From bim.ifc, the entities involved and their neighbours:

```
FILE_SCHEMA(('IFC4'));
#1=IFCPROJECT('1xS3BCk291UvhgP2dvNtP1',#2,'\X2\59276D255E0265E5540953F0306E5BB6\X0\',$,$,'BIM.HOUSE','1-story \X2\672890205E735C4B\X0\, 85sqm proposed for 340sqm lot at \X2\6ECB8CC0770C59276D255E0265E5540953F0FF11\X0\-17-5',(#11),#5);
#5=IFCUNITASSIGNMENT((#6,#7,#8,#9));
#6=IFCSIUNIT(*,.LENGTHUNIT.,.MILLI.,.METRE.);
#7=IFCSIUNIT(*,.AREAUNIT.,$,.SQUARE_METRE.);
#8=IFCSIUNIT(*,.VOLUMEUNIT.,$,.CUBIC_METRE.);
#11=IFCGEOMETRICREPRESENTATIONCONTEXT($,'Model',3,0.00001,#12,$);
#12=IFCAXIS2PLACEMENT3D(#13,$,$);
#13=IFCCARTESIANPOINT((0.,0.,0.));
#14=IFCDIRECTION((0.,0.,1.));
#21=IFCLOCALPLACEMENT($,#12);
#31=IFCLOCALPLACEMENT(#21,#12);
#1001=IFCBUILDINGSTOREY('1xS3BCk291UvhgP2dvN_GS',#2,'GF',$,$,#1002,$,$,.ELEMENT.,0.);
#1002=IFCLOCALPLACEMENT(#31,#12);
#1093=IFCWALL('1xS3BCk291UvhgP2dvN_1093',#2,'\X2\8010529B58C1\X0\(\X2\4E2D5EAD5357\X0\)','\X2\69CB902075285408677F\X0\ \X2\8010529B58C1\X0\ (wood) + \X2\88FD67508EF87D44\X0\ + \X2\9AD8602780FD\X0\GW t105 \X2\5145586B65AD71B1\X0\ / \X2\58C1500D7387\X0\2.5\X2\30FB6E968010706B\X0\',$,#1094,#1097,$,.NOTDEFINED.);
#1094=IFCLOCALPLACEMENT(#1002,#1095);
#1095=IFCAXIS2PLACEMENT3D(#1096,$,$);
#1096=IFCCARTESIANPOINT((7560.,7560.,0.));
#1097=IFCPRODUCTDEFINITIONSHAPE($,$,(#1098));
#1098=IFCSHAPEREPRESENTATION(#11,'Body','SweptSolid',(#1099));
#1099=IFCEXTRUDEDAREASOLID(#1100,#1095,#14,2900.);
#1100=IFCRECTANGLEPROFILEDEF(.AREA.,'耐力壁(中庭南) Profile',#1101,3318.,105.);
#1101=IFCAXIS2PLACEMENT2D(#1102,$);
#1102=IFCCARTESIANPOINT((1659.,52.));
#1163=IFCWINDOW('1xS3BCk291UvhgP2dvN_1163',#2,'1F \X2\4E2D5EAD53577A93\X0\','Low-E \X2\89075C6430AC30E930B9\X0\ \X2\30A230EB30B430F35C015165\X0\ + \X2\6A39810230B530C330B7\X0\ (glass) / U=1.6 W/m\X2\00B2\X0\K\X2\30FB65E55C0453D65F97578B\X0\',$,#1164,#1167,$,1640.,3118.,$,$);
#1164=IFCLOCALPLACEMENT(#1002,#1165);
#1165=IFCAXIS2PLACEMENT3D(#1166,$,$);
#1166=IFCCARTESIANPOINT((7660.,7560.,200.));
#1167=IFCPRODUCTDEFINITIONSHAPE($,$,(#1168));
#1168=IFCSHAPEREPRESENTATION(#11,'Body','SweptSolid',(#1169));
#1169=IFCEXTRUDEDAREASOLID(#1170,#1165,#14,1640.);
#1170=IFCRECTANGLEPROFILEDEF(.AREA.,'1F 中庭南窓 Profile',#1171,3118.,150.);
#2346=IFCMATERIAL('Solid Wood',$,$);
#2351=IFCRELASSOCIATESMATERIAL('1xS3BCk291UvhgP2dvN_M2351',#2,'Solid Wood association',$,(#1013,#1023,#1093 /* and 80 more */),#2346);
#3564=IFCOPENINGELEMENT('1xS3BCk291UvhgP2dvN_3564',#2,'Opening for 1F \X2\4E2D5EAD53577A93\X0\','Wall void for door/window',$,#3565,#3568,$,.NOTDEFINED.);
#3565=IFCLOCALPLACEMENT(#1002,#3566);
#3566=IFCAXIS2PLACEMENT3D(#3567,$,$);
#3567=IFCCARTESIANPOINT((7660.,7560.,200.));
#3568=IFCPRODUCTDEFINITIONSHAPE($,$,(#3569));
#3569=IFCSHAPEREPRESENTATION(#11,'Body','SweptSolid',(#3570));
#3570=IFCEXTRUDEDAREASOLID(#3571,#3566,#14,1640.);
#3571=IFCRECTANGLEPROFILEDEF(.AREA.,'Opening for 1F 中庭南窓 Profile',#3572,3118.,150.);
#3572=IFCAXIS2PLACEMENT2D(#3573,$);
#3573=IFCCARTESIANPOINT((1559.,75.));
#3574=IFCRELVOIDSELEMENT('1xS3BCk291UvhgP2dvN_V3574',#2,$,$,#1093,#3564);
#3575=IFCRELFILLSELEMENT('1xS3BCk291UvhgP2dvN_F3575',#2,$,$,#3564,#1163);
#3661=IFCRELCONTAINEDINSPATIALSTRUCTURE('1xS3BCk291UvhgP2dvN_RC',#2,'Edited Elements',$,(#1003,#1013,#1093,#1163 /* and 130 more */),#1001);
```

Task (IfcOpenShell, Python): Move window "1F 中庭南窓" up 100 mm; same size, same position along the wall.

```python
import numpy as np
import ifcopenshell
import ifcopenshell.api.geometry
import ifcopenshell.util.placement
import ifcopenshell.util.unit

model = ifcopenshell.open("bim.ifc")
unit_scale = ifcopenshell.util.unit.calculate_unit_scale(model)

window = model.by_guid("1xS3BCk291UvhgP2dvN_1163")
opening = window.FillsVoids[0].RelatingOpeningElement
dz = 0.1 / unit_scale

shift = np.array([0.0, 0.0, dz])
# The window is not placed relative to its opening, so move both.
for product in (opening, window):
    matrix = ifcopenshell.util.placement.get_local_placement(product.ObjectPlacement)
    matrix[:3, 3] += shift
    ifcopenshell.api.geometry.edit_object_placement(model, product=product, matrix=matrix, is_si=False)

print(f"moved by {dz * unit_scale:+.3f} m")

model.write("bim_updated.ifc")
```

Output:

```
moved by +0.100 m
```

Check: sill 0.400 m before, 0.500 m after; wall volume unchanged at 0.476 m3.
